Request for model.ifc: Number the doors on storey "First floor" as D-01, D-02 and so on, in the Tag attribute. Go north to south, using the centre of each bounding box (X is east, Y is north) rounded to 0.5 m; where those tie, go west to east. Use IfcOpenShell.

First a look at what the model holds.

```python
import ifcopenshell
import ifcopenshell.util.element
import ifcopenshell.util.placement

model = ifcopenshell.open("model.ifc")
print(model.schema)
storey = next(s for s in model.by_type("IfcBuildingStorey") if s.Name == "First floor")
doors = [e for e in ifcopenshell.util.element.get_decomposition(storey) if e.is_a("IfcDoor")]
for e in sorted(doors, key=lambda e: e.id()):
    origin = ifcopenshell.util.placement.get_local_placement(e.ObjectPlacement)[:3, 3]
    print(e.id(), e.Tag, e.Name, origin.round(2) + 0.0, sep=" | ")
```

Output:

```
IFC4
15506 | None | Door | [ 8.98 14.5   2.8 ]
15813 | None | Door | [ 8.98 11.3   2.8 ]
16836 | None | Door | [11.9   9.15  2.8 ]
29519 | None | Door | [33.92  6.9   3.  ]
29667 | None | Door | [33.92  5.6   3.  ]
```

```python
import ifcopenshell
import ifcopenshell.geom
import ifcopenshell.util.element
import ifcopenshell.util.shape

model = ifcopenshell.open("model.ifc")
settings = ifcopenshell.geom.settings()
settings.set("use-world-coords", True)


def centre(element):
    shape = ifcopenshell.geom.create_shape(settings, element)
    return ifcopenshell.util.shape.get_bbox_centroid(shape.geometry)


storey = next(s for s in model.by_type("IfcBuildingStorey") if s.Name == "First floor")
doors = [e for e in ifcopenshell.util.element.get_decomposition(storey) if e.is_a("IfcDoor")]

# Insertion points can sit at a corner or the storey origin, so sort by the geometry (in metres).
centres = {e: centre(e) for e in doors}
doors.sort(key=lambda e: (-round(centres[e][1] / 0.5), centres[e][0]))

for i, e in enumerate(doors, start=1):
    number = f"D-{i:02d}"
    e.Tag = number
    print(e.id(), number)

model.write("model_updated.ifc")
```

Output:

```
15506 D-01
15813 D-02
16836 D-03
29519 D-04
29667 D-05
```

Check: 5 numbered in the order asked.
